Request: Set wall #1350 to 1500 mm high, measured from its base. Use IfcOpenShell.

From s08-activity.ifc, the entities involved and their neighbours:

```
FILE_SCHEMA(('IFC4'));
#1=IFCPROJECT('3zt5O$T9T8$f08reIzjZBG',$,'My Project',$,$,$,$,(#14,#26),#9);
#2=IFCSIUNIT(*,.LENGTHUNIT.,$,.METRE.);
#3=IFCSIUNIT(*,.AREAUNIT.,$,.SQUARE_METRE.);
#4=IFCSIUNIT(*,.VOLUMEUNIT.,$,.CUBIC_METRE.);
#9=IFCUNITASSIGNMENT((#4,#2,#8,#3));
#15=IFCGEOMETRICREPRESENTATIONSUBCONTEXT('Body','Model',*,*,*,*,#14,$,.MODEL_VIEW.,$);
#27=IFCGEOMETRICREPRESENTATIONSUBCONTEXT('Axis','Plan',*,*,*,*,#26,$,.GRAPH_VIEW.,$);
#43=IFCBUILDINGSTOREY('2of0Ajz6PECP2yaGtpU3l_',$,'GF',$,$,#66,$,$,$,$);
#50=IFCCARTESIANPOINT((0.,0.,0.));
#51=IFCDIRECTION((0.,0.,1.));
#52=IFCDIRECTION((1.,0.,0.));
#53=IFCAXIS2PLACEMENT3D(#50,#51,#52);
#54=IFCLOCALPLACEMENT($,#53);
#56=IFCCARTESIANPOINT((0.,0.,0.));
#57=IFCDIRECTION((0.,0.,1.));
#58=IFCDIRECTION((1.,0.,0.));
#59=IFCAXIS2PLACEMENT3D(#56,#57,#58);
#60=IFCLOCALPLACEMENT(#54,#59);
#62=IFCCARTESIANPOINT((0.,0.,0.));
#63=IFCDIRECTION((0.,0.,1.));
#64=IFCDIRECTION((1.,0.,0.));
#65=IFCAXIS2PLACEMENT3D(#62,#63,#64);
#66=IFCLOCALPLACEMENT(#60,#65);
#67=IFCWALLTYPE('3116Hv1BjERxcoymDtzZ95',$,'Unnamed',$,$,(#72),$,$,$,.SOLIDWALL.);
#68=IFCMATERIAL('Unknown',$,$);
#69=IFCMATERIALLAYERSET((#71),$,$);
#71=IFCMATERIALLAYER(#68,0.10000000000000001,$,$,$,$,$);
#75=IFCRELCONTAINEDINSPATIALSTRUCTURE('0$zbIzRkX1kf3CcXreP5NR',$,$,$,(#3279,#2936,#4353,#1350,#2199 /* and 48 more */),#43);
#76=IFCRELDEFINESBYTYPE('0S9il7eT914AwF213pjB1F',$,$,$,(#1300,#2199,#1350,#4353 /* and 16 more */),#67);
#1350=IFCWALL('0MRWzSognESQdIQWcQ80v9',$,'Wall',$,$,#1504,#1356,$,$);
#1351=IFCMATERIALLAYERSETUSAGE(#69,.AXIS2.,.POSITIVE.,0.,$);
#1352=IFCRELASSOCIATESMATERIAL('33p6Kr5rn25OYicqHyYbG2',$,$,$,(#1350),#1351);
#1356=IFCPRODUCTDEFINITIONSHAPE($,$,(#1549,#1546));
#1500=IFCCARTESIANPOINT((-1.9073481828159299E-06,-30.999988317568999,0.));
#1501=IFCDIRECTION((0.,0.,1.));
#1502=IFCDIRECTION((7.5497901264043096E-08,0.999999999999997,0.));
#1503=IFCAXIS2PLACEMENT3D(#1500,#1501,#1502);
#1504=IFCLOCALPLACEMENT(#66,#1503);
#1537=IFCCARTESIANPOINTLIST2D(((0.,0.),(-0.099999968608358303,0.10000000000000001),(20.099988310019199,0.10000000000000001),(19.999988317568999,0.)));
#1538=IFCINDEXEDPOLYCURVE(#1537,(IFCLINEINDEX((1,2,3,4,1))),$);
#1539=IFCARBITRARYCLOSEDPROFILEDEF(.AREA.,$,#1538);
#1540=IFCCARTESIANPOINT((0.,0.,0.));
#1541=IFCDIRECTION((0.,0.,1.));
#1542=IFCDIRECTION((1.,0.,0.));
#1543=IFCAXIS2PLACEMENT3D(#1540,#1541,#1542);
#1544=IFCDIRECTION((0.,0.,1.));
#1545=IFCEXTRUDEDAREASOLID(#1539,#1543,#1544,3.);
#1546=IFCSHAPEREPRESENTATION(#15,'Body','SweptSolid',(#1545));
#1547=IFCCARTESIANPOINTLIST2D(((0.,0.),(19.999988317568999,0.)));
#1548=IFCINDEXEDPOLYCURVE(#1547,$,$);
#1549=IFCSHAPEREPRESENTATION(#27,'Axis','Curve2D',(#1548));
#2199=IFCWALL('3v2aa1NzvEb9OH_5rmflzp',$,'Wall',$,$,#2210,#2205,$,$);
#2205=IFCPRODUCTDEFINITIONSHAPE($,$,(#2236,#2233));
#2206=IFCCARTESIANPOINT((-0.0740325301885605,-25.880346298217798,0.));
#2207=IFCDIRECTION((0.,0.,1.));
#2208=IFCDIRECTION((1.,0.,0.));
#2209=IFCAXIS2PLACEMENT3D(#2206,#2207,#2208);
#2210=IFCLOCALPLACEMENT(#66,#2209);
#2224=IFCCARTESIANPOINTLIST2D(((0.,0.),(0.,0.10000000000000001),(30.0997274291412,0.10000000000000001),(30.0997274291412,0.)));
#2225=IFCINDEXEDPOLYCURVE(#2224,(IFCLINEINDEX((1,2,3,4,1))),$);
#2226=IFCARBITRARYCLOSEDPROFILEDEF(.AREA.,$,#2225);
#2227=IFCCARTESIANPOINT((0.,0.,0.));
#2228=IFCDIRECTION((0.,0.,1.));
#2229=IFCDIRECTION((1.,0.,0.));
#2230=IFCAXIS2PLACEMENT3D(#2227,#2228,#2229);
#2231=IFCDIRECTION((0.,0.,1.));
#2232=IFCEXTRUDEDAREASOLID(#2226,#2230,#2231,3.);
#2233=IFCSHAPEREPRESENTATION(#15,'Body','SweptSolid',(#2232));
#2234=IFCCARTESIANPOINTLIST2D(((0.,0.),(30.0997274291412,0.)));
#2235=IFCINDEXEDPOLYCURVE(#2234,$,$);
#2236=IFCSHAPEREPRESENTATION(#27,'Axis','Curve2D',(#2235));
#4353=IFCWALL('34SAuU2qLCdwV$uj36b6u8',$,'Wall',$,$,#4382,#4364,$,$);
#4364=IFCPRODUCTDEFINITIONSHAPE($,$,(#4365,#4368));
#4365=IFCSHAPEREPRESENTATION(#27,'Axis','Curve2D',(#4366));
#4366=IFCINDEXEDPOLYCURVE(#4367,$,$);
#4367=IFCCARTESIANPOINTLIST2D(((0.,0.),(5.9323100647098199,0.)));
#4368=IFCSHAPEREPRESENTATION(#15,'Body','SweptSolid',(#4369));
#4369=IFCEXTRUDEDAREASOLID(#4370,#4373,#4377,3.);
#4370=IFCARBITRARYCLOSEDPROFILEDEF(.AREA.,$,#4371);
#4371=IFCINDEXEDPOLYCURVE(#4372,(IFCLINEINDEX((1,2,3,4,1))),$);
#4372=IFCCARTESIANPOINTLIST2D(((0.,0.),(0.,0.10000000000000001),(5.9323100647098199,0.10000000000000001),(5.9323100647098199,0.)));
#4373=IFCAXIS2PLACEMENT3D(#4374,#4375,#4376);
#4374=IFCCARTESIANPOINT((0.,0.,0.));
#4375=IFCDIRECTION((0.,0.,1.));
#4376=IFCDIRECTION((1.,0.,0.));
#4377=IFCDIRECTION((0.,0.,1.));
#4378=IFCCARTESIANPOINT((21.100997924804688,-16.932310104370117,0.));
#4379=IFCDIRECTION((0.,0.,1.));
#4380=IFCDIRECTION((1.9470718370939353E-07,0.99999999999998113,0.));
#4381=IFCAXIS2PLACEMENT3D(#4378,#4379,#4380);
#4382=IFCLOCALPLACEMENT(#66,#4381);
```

```python
import ifcopenshell
import ifcopenshell.geom
import ifcopenshell.util.representation
import ifcopenshell.util.shape

model = ifcopenshell.open("s08-activity.ifc")
settings = ifcopenshell.geom.settings()


def volume(element):
    """Net volume in cubic metres, openings subtracted."""
    shape = ifcopenshell.geom.create_shape(settings, element)
    return ifcopenshell.util.shape.get_volume(shape.geometry)


wall = model.by_guid("0MRWzSognESQdIQWcQ80v9")
before = volume(wall)

body = ifcopenshell.util.representation.get_representation(wall, "Model", "Body")
solid = body.Items[0]
old_height = solid.Depth
solid.Depth = 1.5
after = volume(wall)

print(f"height {old_height:g} -> {solid.Depth:g}, volume {before:.3f} -> {after:.3f} m3")

model.write("s08-activity_edited.ifc")
```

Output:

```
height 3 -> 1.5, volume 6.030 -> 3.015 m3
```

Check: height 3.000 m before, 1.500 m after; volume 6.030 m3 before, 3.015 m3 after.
